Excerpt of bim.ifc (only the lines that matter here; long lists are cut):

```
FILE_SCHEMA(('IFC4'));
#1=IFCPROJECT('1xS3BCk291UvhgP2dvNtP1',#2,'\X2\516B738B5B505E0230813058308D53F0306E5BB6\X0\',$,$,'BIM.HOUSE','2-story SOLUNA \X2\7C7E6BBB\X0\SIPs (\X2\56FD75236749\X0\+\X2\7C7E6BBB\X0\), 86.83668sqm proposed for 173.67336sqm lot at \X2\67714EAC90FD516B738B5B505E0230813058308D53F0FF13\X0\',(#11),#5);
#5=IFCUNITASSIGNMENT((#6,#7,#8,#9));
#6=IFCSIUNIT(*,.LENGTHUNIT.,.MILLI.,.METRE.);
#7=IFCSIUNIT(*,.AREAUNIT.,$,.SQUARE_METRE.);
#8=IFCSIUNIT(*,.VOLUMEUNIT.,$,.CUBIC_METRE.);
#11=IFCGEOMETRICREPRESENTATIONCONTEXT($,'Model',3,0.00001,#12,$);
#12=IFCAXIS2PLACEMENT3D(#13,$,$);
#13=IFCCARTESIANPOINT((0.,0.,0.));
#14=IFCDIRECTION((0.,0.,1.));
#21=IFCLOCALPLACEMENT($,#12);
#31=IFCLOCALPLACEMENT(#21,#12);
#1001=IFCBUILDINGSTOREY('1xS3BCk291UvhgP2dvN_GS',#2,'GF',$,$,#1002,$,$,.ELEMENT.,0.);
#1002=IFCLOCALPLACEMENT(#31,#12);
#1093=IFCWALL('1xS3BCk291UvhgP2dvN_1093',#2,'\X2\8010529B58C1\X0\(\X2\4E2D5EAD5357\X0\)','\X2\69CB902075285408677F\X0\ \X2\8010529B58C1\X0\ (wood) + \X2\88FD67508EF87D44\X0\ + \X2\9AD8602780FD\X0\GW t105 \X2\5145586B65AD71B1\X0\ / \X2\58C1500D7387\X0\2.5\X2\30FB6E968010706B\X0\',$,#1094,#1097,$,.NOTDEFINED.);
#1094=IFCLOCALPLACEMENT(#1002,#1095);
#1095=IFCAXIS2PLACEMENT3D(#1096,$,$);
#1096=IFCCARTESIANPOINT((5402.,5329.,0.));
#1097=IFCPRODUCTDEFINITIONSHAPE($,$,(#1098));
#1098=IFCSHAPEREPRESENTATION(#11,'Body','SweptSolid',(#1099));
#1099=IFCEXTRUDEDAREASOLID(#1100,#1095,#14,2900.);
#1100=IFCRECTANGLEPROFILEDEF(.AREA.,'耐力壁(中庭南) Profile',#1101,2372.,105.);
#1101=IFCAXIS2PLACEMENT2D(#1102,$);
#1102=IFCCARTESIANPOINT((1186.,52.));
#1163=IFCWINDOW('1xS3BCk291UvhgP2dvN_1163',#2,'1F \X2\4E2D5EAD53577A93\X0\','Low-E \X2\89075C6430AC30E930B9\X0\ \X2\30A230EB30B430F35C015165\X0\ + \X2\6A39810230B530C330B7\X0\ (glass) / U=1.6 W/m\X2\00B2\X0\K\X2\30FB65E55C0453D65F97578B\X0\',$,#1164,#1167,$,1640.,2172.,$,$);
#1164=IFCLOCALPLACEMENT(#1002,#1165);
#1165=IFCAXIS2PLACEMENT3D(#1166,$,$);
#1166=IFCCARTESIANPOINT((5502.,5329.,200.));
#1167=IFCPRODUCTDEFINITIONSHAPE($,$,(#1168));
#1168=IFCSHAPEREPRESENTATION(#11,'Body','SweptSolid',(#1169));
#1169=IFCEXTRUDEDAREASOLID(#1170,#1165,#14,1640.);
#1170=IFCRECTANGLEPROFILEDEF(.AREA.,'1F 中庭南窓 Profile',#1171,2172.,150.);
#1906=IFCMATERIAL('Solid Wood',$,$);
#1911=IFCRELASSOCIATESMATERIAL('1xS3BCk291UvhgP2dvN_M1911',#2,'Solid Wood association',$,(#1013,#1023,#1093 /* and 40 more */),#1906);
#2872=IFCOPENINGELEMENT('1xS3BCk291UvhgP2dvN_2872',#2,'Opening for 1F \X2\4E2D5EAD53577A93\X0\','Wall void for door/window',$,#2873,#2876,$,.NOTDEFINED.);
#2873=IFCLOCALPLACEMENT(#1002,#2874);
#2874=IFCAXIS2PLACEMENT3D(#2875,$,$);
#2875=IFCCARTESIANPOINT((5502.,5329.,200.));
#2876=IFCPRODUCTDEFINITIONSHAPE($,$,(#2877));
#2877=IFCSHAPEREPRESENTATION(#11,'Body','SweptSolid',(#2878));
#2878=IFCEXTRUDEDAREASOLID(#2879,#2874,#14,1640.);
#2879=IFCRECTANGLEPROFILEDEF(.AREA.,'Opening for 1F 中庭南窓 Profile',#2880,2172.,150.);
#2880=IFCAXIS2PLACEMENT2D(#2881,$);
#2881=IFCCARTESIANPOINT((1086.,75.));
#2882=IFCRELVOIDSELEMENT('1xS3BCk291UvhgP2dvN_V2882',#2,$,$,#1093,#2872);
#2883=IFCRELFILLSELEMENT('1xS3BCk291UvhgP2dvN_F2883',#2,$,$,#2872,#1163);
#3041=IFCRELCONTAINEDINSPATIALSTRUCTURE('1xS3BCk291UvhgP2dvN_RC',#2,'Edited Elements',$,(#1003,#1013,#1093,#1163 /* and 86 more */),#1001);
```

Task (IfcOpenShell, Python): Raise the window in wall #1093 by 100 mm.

```python
import numpy as np
import ifcopenshell
import ifcopenshell.api.geometry
import ifcopenshell.util.placement
import ifcopenshell.util.unit

model = ifcopenshell.open("bim.ifc")
unit_scale = ifcopenshell.util.unit.calculate_unit_scale(model)

window = model.by_guid("1xS3BCk291UvhgP2dvN_1163")
opening = window.FillsVoids[0].RelatingOpeningElement
dz = 100.0

shift = np.array([0.0, 0.0, dz])
# The window is not placed relative to its opening, so move both.
for product in (opening, window):
    matrix = ifcopenshell.util.placement.get_local_placement(product.ObjectPlacement)
    matrix[:3, 3] += shift
    ifcopenshell.api.geometry.edit_object_placement(model, product=product, matrix=matrix, is_si=False)

print(f"moved by {dz * unit_scale:+.3f} m")

model.write("bim_v2.ifc")
```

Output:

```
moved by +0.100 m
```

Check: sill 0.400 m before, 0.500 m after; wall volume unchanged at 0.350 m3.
